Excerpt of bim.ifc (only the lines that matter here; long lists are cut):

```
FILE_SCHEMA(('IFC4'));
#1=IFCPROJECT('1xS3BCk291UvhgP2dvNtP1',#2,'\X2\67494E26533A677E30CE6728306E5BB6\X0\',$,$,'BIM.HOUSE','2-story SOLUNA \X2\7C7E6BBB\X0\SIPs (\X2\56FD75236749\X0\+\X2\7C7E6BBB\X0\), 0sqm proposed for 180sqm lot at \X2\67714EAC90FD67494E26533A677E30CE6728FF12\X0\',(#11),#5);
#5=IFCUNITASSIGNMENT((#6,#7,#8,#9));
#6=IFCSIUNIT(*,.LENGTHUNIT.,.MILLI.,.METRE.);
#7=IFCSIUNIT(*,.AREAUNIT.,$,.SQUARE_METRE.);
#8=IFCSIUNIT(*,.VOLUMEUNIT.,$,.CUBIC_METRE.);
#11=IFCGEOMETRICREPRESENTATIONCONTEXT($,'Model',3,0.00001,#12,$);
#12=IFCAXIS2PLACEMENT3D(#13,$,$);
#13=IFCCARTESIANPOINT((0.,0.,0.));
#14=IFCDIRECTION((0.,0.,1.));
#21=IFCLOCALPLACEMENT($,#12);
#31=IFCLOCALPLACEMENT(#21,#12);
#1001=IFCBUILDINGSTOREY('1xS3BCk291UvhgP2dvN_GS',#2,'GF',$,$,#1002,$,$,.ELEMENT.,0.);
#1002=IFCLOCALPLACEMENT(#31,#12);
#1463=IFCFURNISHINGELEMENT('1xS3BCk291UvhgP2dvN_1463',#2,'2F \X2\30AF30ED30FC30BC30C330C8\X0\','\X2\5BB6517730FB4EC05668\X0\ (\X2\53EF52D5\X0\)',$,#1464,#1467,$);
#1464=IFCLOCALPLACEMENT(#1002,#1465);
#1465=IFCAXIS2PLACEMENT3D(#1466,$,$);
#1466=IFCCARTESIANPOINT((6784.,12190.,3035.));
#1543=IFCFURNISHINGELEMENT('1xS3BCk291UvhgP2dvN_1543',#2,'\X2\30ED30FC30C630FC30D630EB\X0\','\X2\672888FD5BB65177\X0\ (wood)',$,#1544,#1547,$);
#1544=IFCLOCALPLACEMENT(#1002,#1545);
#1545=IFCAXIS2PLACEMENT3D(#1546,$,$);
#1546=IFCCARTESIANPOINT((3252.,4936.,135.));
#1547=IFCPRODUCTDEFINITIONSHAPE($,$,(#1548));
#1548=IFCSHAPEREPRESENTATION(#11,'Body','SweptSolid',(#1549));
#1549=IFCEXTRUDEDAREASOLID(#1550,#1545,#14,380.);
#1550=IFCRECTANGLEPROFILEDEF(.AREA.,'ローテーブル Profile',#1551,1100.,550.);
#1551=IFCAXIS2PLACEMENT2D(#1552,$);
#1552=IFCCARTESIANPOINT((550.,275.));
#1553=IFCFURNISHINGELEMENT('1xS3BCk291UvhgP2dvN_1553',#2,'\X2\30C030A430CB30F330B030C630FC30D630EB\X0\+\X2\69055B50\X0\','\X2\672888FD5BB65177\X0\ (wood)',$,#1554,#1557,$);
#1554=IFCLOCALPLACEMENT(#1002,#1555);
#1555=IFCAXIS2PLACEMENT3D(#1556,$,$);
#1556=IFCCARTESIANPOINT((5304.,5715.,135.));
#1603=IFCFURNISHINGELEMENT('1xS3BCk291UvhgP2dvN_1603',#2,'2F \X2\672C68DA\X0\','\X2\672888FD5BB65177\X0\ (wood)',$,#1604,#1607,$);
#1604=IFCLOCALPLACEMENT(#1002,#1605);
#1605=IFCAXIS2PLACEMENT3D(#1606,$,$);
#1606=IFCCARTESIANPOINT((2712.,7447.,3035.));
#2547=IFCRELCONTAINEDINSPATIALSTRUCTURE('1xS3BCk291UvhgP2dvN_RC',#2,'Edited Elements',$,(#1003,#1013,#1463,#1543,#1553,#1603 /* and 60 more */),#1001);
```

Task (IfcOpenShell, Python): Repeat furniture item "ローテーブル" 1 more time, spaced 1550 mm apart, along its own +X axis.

```python
import ifcopenshell
import ifcopenshell.api.geometry
import ifcopenshell.api.root
import ifcopenshell.util.element
import ifcopenshell.util.placement
import ifcopenshell.util.unit

model = ifcopenshell.open("bim.ifc")
unit_scale = ifcopenshell.util.unit.calculate_unit_scale(model)


def reuse_history(source, copy):
    """copy_class also copies each property set's owner history, people and application; keep the originals."""
    for rel in copy.IsDefinedBy:
        if rel.is_a("IfcRelDefinesByProperties") and (history := rel.RelatingPropertyDefinition.OwnerHistory):
            rel.RelatingPropertyDefinition.OwnerHistory = source.OwnerHistory
            ifcopenshell.util.element.remove_deep2(model, history)


source = model.by_guid("1xS3BCk291UvhgP2dvN_1543")
base = ifcopenshell.util.placement.get_local_placement(source.ObjectPlacement)
step = base[:3, 0] * 1.55 / unit_scale

for i in range(1, 2):
    copy = ifcopenshell.api.root.copy_class(model, product=source)
    copy.Representation = ifcopenshell.util.element.copy_deep(
        model, source.Representation, exclude=["IfcGeometricRepresentationContext", "IfcRepresentationMap"]
    )
    reuse_history(source, copy)
    matrix = base.copy()
    matrix[:3, 3] += i * step
    print("added at", matrix[:3, 3].round(3) + 0.0)
    ifcopenshell.api.geometry.edit_object_placement(model, product=copy, matrix=matrix, is_si=False)

model.write("bim_rev.ifc")
```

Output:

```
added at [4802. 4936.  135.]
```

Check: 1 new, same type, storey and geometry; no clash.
